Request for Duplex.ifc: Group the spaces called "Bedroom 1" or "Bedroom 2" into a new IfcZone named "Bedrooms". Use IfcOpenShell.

First a look at what the model holds.

```python
import ifcopenshell

model = ifcopenshell.open("Duplex.ifc")
print(model.schema)
seen = {}
for space in model.by_type("IfcSpace"):
    seen[space.LongName] = seen.get(space.LongName, 0) + 1
for name, count in sorted(seen.items(), key=str):
    print(count, "x", name)
print("zones:", [z.Name for z in model.by_type("IfcZone")][:20])
```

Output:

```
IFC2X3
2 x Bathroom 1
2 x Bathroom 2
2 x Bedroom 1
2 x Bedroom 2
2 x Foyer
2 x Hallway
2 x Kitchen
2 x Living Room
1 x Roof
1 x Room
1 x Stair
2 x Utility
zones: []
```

```python
import ifcopenshell
import ifcopenshell.api.group
import ifcopenshell.api.root

model = ifcopenshell.open("Duplex.ifc")

names = {"Bedroom 1", "Bedroom 2"}
spaces = [s for s in model.by_type("IfcSpace") if s.LongName in names]

zone = ifcopenshell.api.root.create_entity(model, ifc_class="IfcZone", name="Bedrooms")
ifcopenshell.api.group.assign_group(model, products=spaces, group=zone)
print(len(spaces), "spaces in", zone.Name)

model.write("Duplex_edited.ifc")
```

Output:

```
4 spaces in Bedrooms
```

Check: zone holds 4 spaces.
